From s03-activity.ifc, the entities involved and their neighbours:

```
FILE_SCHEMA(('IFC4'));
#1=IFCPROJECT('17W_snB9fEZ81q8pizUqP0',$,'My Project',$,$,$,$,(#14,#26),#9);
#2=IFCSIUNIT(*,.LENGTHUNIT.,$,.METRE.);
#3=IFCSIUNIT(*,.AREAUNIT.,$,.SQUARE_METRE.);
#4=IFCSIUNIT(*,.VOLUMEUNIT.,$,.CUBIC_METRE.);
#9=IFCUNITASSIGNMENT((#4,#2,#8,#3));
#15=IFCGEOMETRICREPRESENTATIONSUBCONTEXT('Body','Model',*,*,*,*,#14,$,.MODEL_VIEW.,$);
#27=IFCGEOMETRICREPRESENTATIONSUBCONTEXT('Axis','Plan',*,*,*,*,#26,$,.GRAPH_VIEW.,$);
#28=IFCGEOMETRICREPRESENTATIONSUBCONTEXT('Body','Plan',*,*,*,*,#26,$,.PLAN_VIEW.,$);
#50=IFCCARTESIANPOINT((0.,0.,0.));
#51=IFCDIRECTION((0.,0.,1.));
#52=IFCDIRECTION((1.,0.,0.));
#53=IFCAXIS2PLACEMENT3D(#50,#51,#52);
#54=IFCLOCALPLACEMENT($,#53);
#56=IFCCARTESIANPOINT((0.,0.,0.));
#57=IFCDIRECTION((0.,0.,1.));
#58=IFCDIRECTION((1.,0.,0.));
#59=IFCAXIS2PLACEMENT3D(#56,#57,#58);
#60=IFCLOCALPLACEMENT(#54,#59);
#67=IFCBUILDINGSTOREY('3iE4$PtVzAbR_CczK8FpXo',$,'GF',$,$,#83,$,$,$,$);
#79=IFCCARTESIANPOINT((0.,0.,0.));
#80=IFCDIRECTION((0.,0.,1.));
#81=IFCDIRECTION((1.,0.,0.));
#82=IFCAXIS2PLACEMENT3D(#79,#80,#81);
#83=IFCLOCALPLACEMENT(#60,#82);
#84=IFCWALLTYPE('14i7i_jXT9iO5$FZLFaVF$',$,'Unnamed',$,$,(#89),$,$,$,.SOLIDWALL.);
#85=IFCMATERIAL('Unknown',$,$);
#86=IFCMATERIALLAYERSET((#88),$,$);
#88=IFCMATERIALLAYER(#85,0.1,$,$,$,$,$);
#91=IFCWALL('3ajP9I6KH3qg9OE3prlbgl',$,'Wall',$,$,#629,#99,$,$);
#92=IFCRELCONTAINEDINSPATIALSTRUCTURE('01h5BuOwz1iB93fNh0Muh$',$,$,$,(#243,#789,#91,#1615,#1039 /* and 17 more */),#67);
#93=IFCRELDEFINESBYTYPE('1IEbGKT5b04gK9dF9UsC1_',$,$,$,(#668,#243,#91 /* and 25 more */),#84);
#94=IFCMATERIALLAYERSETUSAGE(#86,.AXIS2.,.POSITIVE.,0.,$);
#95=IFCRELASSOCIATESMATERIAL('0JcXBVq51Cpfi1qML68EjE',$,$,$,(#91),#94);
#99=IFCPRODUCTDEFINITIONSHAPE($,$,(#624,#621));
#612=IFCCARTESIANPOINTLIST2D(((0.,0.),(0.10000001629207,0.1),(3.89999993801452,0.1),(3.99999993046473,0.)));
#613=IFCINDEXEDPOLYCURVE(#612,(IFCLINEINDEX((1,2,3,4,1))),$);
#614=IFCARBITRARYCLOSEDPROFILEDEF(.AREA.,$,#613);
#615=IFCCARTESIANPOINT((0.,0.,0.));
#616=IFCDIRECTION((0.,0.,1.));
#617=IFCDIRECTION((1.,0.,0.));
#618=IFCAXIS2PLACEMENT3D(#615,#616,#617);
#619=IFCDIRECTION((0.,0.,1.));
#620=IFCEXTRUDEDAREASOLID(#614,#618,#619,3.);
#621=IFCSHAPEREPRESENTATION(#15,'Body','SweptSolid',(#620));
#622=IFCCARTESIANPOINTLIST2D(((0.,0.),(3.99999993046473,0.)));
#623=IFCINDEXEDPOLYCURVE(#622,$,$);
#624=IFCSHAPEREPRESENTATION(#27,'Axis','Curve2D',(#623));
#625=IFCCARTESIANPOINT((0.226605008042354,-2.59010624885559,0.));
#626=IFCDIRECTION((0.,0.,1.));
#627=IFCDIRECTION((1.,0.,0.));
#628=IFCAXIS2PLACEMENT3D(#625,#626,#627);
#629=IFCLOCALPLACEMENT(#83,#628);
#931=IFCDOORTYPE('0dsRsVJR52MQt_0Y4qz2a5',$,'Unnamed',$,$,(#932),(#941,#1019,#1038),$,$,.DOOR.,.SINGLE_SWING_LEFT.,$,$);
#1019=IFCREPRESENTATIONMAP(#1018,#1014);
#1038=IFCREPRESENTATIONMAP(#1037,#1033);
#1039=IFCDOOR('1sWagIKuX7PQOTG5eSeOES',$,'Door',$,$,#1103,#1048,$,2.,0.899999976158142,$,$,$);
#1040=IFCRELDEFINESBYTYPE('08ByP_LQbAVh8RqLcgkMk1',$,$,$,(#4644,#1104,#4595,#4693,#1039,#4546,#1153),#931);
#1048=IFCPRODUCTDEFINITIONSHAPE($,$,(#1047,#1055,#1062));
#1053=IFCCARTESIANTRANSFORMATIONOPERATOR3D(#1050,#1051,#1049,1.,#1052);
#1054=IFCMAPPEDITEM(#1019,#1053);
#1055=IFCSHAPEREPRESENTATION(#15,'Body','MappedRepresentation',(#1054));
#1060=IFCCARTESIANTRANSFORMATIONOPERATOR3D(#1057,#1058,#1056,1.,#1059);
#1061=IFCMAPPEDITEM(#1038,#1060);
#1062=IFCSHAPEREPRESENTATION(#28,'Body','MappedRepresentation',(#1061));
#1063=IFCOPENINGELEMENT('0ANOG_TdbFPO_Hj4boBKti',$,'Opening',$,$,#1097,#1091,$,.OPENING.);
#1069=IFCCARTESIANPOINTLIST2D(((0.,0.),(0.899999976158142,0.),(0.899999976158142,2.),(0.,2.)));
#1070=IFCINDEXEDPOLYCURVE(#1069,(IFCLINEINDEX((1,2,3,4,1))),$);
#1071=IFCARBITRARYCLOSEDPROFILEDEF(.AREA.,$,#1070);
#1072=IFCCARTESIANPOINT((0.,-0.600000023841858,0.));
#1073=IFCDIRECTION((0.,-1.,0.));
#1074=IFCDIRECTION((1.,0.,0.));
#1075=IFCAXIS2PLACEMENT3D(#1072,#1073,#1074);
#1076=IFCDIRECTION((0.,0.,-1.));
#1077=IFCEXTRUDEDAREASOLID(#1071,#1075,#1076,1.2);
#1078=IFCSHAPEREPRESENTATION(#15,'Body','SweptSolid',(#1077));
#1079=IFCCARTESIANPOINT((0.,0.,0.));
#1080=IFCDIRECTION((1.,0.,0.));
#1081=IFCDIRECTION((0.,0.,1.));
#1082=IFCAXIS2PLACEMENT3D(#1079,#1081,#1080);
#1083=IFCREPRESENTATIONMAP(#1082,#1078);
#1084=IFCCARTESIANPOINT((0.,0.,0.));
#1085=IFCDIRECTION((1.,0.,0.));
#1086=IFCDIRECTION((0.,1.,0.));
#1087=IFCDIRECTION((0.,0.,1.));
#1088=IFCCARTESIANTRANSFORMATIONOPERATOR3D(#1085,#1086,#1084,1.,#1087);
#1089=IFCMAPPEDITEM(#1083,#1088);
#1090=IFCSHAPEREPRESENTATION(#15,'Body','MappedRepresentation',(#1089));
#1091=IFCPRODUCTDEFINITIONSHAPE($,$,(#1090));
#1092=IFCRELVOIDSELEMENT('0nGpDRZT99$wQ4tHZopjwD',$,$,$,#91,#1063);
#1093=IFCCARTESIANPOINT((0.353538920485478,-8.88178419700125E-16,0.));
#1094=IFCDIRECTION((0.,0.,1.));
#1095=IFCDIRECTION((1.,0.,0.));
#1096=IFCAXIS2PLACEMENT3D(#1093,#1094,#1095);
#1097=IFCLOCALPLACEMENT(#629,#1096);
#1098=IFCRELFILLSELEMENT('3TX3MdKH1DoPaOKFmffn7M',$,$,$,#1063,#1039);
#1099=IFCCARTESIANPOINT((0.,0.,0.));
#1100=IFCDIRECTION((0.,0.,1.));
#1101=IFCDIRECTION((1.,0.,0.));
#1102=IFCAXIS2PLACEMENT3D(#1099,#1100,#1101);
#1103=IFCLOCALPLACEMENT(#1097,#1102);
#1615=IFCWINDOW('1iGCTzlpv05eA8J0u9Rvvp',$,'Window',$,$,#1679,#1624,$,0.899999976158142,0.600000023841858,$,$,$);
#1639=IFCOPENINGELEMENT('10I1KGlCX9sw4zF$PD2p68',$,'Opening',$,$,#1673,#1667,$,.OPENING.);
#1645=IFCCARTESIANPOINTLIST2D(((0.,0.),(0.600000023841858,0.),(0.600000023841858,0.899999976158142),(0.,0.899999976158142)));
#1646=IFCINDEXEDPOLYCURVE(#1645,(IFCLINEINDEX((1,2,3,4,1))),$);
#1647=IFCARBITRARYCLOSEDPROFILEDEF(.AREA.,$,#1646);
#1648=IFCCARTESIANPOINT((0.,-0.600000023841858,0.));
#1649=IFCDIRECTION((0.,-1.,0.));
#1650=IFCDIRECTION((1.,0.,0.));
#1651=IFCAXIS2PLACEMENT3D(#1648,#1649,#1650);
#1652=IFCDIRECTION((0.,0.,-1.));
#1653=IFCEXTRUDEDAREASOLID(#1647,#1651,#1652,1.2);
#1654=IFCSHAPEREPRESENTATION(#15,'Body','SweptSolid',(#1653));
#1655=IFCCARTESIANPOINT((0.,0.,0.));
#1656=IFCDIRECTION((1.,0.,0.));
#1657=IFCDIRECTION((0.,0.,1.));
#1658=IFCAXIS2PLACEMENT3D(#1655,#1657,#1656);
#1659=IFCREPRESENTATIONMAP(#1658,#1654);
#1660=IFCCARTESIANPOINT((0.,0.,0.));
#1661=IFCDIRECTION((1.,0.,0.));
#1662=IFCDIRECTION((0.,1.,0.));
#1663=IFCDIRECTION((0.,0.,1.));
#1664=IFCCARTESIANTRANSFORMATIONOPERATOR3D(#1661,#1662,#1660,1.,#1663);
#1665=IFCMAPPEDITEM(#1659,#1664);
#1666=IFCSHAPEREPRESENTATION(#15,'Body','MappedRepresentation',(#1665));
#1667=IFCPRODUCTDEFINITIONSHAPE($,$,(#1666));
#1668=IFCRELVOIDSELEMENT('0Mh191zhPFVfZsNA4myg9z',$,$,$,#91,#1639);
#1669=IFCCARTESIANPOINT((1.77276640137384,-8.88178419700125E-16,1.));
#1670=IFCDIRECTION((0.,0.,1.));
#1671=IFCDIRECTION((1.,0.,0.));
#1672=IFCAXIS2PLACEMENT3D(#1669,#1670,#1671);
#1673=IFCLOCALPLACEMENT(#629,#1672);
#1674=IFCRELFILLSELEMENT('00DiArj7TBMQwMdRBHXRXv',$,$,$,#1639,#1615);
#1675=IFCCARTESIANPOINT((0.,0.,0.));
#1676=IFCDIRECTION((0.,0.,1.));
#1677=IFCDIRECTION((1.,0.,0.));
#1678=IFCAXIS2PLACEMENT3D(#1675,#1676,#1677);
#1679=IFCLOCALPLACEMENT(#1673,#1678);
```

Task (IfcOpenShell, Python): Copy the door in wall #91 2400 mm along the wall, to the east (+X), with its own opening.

```python
import ifcopenshell
import ifcopenshell.api.feature
import ifcopenshell.api.geometry
import ifcopenshell.api.root
import ifcopenshell.geom
import ifcopenshell.util.element
import ifcopenshell.util.placement
import ifcopenshell.util.shape
import ifcopenshell.util.unit

model = ifcopenshell.open("s03-activity.ifc")
unit_scale = ifcopenshell.util.unit.calculate_unit_scale(model)
settings = ifcopenshell.geom.settings()


def volume(element):
    """Net volume in cubic metres, openings subtracted."""
    shape = ifcopenshell.geom.create_shape(settings, element)
    return ifcopenshell.util.shape.get_volume(shape.geometry)


door = model.by_guid("1sWagIKuX7PQOTG5eSeOES")
opening = door.FillsVoids[0].RelatingOpeningElement
wall = opening.VoidsElements[0].RelatingBuildingElement
before = volume(wall)
shift = ifcopenshell.util.placement.get_local_placement(wall.ObjectPlacement)[:3, 0] * 2.4 / unit_scale

# copy_class copies the void relationship, type, container and properties, but no geometry.
new_opening = ifcopenshell.api.root.copy_class(model, product=opening)
new_opening.Representation = ifcopenshell.util.element.copy_deep(
    model, opening.Representation, exclude=["IfcGeometricRepresentationContext", "IfcRepresentationMap"]
)
new_door = ifcopenshell.api.root.copy_class(model, product=door)
new_door.Representation = ifcopenshell.util.element.copy_deep(
    model, door.Representation, exclude=["IfcGeometricRepresentationContext", "IfcRepresentationMap"]
)
ifcopenshell.api.feature.add_filling(model, opening=new_opening, element=new_door)

for old, new in ((opening, new_opening), (door, new_door)):
    matrix = ifcopenshell.util.placement.get_local_placement(old.ObjectPlacement)
    matrix[:3, 3] += shift
    ifcopenshell.api.geometry.edit_object_placement(model, product=new, matrix=matrix, is_si=False)

after = volume(wall)

print(f"wall volume {before:.3f} -> {after:.3f} m3")

model.write("s03-activity_updated.ifc")
```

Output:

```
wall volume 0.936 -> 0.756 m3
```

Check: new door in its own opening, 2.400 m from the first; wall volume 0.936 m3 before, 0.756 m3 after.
